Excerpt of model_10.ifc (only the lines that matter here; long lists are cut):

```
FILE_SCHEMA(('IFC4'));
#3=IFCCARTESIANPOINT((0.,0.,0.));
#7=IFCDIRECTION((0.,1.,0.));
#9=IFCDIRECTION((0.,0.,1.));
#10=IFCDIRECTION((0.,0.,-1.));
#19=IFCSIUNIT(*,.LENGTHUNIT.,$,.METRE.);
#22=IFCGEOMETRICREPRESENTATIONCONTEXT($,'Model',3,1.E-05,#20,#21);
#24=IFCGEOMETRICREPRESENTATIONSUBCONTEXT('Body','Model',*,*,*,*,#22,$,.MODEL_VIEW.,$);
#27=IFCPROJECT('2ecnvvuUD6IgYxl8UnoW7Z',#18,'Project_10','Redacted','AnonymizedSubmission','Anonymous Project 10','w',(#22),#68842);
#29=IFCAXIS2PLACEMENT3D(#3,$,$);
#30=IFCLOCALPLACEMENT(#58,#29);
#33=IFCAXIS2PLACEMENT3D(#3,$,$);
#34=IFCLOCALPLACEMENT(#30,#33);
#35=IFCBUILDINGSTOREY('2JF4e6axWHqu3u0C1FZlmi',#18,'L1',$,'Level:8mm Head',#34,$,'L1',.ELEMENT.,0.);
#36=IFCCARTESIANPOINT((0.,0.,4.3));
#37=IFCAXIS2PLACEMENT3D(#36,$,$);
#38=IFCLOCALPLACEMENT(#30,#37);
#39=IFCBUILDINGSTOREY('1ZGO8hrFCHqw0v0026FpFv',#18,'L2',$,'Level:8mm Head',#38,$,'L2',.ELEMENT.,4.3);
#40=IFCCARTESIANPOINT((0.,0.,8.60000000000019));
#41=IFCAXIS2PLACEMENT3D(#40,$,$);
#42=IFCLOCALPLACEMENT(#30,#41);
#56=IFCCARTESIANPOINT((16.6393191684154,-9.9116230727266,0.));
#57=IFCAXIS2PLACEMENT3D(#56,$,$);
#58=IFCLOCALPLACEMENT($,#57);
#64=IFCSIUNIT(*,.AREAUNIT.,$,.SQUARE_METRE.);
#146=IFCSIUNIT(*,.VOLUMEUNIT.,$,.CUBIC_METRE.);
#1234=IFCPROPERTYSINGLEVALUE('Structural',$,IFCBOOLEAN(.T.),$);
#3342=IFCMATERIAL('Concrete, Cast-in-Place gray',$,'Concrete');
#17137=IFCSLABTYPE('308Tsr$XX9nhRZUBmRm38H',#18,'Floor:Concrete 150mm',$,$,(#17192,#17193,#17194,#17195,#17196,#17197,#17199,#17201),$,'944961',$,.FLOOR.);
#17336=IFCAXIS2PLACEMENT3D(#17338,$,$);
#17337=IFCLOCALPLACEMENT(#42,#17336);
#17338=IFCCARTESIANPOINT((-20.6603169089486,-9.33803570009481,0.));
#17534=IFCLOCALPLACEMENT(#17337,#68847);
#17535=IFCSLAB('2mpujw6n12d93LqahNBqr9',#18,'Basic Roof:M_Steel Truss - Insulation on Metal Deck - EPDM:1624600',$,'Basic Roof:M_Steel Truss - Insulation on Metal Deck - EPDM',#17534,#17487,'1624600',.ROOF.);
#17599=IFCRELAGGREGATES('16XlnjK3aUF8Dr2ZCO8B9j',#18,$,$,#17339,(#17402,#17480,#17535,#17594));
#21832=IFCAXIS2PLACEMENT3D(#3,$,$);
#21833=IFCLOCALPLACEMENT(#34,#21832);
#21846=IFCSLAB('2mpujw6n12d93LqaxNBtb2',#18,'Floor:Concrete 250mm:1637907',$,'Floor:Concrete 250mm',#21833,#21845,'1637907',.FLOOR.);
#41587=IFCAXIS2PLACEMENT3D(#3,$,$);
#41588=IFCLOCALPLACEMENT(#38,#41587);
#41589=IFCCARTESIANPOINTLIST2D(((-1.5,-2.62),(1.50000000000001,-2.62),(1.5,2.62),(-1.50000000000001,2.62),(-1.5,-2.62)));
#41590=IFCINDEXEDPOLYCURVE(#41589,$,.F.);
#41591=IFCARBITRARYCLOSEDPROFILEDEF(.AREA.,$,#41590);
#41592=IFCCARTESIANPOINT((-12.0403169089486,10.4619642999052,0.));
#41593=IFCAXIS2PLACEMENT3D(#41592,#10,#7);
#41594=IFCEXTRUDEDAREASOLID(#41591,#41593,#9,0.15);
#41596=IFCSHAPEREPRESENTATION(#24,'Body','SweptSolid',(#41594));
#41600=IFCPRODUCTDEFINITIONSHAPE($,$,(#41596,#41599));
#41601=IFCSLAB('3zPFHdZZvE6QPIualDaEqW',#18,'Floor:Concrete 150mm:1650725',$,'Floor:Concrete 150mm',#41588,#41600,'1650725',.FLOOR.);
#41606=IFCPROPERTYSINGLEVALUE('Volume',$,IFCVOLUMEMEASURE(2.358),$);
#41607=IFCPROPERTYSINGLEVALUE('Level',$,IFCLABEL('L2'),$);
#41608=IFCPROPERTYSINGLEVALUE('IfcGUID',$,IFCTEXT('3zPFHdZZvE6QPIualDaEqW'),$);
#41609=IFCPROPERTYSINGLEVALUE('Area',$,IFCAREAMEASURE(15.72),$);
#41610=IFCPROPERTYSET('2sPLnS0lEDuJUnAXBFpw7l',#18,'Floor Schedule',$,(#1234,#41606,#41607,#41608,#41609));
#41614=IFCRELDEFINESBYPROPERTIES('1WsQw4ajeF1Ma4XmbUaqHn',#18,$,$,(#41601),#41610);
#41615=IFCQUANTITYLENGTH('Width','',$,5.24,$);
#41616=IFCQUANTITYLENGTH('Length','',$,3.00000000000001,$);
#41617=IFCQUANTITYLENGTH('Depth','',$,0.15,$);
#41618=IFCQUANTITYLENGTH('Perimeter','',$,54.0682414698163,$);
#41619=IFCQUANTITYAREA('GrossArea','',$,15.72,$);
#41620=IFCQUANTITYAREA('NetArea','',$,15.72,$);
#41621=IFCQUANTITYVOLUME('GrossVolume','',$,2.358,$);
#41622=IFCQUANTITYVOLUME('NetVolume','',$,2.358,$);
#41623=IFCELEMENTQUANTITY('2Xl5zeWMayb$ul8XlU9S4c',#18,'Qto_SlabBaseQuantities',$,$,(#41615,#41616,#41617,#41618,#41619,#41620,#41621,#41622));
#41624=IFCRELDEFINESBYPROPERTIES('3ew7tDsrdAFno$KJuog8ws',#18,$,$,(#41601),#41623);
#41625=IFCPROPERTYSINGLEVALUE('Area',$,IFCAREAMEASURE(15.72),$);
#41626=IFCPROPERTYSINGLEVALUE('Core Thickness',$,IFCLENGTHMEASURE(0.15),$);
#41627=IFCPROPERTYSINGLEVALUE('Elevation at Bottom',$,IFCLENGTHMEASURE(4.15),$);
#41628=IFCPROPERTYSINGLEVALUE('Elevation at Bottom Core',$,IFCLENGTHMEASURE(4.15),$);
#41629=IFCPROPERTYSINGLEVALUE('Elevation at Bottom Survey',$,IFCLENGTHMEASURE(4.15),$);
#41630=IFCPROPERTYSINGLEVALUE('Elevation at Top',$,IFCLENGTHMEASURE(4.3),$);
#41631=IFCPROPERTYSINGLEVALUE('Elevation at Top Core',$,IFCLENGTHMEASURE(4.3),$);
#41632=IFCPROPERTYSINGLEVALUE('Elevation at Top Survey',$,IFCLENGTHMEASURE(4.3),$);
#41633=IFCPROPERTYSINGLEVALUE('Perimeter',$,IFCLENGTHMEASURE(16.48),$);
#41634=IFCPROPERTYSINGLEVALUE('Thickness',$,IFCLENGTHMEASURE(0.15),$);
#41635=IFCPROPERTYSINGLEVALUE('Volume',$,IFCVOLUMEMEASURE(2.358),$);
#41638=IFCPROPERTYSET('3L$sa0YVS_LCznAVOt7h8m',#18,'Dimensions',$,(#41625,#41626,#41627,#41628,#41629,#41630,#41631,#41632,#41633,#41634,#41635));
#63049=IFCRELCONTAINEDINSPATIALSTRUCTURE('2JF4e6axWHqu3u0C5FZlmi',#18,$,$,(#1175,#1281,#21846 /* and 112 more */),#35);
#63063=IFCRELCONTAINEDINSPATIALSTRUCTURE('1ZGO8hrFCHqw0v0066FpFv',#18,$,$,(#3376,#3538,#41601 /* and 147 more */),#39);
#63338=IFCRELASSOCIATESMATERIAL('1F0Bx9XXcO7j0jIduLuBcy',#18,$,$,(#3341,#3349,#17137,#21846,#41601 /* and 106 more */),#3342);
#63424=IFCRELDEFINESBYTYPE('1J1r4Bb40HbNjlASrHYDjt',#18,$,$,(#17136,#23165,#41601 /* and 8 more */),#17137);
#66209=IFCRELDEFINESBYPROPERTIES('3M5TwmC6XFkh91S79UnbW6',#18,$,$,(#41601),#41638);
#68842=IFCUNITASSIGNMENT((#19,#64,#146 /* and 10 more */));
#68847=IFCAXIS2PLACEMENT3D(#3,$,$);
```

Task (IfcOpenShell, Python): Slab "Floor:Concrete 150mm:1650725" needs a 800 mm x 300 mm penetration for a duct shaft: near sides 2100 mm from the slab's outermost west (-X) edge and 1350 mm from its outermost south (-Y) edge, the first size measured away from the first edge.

```python
import numpy as np
import ifcopenshell
import ifcopenshell.api.feature
import ifcopenshell.api.geometry
import ifcopenshell.api.pset
import ifcopenshell.api.root
import ifcopenshell.geom
import ifcopenshell.util.element
import ifcopenshell.util.placement
import ifcopenshell.util.representation
import ifcopenshell.util.shape
import ifcopenshell.util.unit

model = ifcopenshell.open("model_10.ifc")
unit_scale = ifcopenshell.util.unit.calculate_unit_scale(model)
area_scale = ifcopenshell.util.unit.calculate_unit_scale(model, "AREAUNIT")
volume_scale = ifcopenshell.util.unit.calculate_unit_scale(model, "VOLUMEUNIT")
settings = ifcopenshell.geom.settings()


def volume(element):
    """Net volume in cubic metres, openings subtracted."""
    shape = ifcopenshell.geom.create_shape(settings, element)
    return ifcopenshell.util.shape.get_volume(shape.geometry)


slab = model.by_id(41601)
before = volume(slab)

# Extent in the slab's own axes, in metres. The edges named are its -X and -Y sides.
slab_shape = ifcopenshell.geom.create_shape(settings, slab)
vertices = ifcopenshell.util.shape.get_vertices(slab_shape.geometry)
x_min, y_min, bottom = vertices.min(axis=0)
top = vertices[:, 2].max()

opening = ifcopenshell.api.root.create_entity(model, ifc_class="IfcOpeningElement", name="Duct shaft opening", predefined_type="OPENING")
context = ifcopenshell.util.representation.get_context(model, "Model", "Body", "MODEL_VIEW")
width, depth = 0.8, 0.3
outline = [(0.0, 0.0), (width, 0.0), (width, depth), (0.0, depth), (0.0, 0.0)]
# Overshoot both faces by 50 mm so the cut is clean.
shape = ifcopenshell.api.geometry.add_slab_representation(
    model, context=context, depth=top - bottom + 0.1, polyline=outline
)
ifcopenshell.api.geometry.assign_representation(model, product=opening, representation=shape)

matrix = ifcopenshell.util.placement.get_local_placement(slab.ObjectPlacement)
matrix[:, 3] = matrix @ np.append(np.array([x_min + 2.1, y_min + 1.35, bottom - 0.05]) / unit_scale, 1.0)
ifcopenshell.api.geometry.edit_object_placement(model, product=opening, matrix=matrix, is_si=False)
ifcopenshell.api.feature.add_feature(model, feature=opening, element=slab)

after = volume(slab)

# Update the slab's stored quantities.
pset = model.by_id(ifcopenshell.util.element.get_pset(slab, "Floor Schedule", should_inherit=False)["id"])
ifcopenshell.api.pset.edit_pset(model, pset=pset, properties={
    "Volume": model.create_entity("IfcVolumeMeasure", after / volume_scale),
    "Area": model.create_entity("IfcAreaMeasure", after / (top - bottom) / area_scale),
})
qto = model.by_id(ifcopenshell.util.element.get_pset(slab, "Qto_SlabBaseQuantities", should_inherit=False)["id"])
ifcopenshell.api.pset.edit_qto(model, qto=qto, properties={
    "NetArea": after / (top - bottom) / area_scale,
    "NetVolume": after / volume_scale,
})
pset = model.by_id(ifcopenshell.util.element.get_pset(slab, "Dimensions", should_inherit=False)["id"])
ifcopenshell.api.pset.edit_pset(model, pset=pset, properties={
    "Area": model.create_entity("IfcAreaMeasure", after / (top - bottom) / area_scale),
    "Volume": model.create_entity("IfcVolumeMeasure", after / volume_scale),
})

print(f"slab volume {before:.3f} -> {after:.3f} m3")

model.write("model_10_updated.ifc")
```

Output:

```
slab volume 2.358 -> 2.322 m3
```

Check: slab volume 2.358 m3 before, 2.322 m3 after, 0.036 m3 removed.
